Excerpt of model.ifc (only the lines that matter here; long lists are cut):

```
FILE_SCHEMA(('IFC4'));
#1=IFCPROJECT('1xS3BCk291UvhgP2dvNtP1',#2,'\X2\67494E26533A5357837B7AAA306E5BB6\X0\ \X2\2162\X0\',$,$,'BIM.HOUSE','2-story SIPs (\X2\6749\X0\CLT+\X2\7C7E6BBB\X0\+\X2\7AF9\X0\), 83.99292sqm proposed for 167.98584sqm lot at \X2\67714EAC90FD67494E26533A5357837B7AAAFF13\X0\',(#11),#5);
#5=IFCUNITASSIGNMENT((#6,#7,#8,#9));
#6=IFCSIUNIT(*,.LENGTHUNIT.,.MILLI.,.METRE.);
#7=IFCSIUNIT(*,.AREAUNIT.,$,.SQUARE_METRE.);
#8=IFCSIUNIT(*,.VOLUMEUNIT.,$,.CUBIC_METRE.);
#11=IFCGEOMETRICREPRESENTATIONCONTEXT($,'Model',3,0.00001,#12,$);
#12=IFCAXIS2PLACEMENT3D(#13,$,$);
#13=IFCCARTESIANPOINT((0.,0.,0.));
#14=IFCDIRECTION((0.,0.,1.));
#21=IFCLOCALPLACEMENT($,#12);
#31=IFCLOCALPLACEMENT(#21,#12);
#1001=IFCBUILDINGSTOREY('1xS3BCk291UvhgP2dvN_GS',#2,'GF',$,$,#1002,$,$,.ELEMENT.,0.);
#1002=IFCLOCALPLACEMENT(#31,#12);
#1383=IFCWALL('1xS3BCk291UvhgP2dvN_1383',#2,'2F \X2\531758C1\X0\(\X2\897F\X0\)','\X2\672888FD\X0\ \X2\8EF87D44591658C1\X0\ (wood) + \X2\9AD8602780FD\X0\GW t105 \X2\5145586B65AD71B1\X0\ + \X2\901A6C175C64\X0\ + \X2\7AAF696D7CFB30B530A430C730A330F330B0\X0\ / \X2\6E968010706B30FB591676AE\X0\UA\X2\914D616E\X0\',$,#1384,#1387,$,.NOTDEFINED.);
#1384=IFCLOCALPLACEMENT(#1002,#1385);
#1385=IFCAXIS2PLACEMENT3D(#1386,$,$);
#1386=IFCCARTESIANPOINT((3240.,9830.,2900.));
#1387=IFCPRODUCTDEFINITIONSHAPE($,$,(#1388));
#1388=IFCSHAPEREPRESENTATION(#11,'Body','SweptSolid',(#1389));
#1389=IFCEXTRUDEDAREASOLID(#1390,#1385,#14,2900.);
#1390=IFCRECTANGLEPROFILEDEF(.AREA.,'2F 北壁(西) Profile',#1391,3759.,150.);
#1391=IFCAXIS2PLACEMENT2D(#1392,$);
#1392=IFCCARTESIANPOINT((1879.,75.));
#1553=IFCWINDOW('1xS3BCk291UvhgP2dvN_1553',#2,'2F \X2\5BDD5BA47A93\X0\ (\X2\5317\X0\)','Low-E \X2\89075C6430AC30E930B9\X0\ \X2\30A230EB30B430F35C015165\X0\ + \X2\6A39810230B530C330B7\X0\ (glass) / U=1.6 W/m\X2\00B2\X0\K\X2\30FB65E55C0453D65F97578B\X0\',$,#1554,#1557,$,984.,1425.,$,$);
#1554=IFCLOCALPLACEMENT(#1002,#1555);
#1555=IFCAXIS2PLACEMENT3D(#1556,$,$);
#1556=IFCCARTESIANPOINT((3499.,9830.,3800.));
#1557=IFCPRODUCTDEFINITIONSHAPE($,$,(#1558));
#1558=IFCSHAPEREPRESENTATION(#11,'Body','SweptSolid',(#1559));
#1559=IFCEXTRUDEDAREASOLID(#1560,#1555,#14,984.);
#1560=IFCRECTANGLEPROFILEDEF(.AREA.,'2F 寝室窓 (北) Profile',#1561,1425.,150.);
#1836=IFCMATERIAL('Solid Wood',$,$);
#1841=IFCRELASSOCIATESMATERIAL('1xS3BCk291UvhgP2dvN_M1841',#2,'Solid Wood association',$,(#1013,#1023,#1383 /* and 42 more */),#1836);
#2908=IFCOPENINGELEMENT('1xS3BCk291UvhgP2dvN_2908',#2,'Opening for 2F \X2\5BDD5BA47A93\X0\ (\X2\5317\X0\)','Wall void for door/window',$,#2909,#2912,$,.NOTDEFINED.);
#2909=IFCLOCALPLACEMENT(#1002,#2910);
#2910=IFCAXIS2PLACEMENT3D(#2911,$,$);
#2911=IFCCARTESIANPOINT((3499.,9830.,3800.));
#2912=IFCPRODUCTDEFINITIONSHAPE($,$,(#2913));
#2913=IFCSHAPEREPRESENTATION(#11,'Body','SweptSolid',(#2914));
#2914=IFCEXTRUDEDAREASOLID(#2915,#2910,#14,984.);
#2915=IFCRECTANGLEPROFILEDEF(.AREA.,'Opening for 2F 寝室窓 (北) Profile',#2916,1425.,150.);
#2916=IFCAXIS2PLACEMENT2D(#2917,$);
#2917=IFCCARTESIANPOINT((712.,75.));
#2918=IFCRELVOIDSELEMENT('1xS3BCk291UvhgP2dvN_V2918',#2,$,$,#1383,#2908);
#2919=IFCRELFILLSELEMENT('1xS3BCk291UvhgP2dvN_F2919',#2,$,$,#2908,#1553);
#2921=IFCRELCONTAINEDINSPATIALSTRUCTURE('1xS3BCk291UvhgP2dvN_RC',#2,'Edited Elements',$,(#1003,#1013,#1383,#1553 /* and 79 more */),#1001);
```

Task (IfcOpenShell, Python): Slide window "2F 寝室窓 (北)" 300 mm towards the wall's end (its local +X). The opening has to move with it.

```python
import ifcopenshell
import ifcopenshell.api.geometry
import ifcopenshell.util.placement
import ifcopenshell.util.unit

model = ifcopenshell.open("model.ifc")
unit_scale = ifcopenshell.util.unit.calculate_unit_scale(model)

window = model.by_guid("1xS3BCk291UvhgP2dvN_1553")
opening = window.FillsVoids[0].RelatingOpeningElement
wall = opening.VoidsElements[0].RelatingBuildingElement

wall_matrix = ifcopenshell.util.placement.get_local_placement(wall.ObjectPlacement)
shift = wall_matrix[:3, 0] * 0.3 / unit_scale
before = ifcopenshell.util.placement.get_local_placement(window.ObjectPlacement)[:3, 3].copy()

# The window is not placed relative to its opening, so move both.
for product in (opening, window):
    matrix = ifcopenshell.util.placement.get_local_placement(product.ObjectPlacement)
    matrix[:3, 3] += shift
    ifcopenshell.api.geometry.edit_object_placement(model, product=product, matrix=matrix, is_si=False)

after = ifcopenshell.util.placement.get_local_placement(window.ObjectPlacement)[:3, 3]
print("window moved by", (after - before).round(3) + 0.0)

model.write("model_updated.ifc")
```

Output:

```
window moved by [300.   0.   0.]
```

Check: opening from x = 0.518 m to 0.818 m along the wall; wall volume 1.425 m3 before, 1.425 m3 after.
